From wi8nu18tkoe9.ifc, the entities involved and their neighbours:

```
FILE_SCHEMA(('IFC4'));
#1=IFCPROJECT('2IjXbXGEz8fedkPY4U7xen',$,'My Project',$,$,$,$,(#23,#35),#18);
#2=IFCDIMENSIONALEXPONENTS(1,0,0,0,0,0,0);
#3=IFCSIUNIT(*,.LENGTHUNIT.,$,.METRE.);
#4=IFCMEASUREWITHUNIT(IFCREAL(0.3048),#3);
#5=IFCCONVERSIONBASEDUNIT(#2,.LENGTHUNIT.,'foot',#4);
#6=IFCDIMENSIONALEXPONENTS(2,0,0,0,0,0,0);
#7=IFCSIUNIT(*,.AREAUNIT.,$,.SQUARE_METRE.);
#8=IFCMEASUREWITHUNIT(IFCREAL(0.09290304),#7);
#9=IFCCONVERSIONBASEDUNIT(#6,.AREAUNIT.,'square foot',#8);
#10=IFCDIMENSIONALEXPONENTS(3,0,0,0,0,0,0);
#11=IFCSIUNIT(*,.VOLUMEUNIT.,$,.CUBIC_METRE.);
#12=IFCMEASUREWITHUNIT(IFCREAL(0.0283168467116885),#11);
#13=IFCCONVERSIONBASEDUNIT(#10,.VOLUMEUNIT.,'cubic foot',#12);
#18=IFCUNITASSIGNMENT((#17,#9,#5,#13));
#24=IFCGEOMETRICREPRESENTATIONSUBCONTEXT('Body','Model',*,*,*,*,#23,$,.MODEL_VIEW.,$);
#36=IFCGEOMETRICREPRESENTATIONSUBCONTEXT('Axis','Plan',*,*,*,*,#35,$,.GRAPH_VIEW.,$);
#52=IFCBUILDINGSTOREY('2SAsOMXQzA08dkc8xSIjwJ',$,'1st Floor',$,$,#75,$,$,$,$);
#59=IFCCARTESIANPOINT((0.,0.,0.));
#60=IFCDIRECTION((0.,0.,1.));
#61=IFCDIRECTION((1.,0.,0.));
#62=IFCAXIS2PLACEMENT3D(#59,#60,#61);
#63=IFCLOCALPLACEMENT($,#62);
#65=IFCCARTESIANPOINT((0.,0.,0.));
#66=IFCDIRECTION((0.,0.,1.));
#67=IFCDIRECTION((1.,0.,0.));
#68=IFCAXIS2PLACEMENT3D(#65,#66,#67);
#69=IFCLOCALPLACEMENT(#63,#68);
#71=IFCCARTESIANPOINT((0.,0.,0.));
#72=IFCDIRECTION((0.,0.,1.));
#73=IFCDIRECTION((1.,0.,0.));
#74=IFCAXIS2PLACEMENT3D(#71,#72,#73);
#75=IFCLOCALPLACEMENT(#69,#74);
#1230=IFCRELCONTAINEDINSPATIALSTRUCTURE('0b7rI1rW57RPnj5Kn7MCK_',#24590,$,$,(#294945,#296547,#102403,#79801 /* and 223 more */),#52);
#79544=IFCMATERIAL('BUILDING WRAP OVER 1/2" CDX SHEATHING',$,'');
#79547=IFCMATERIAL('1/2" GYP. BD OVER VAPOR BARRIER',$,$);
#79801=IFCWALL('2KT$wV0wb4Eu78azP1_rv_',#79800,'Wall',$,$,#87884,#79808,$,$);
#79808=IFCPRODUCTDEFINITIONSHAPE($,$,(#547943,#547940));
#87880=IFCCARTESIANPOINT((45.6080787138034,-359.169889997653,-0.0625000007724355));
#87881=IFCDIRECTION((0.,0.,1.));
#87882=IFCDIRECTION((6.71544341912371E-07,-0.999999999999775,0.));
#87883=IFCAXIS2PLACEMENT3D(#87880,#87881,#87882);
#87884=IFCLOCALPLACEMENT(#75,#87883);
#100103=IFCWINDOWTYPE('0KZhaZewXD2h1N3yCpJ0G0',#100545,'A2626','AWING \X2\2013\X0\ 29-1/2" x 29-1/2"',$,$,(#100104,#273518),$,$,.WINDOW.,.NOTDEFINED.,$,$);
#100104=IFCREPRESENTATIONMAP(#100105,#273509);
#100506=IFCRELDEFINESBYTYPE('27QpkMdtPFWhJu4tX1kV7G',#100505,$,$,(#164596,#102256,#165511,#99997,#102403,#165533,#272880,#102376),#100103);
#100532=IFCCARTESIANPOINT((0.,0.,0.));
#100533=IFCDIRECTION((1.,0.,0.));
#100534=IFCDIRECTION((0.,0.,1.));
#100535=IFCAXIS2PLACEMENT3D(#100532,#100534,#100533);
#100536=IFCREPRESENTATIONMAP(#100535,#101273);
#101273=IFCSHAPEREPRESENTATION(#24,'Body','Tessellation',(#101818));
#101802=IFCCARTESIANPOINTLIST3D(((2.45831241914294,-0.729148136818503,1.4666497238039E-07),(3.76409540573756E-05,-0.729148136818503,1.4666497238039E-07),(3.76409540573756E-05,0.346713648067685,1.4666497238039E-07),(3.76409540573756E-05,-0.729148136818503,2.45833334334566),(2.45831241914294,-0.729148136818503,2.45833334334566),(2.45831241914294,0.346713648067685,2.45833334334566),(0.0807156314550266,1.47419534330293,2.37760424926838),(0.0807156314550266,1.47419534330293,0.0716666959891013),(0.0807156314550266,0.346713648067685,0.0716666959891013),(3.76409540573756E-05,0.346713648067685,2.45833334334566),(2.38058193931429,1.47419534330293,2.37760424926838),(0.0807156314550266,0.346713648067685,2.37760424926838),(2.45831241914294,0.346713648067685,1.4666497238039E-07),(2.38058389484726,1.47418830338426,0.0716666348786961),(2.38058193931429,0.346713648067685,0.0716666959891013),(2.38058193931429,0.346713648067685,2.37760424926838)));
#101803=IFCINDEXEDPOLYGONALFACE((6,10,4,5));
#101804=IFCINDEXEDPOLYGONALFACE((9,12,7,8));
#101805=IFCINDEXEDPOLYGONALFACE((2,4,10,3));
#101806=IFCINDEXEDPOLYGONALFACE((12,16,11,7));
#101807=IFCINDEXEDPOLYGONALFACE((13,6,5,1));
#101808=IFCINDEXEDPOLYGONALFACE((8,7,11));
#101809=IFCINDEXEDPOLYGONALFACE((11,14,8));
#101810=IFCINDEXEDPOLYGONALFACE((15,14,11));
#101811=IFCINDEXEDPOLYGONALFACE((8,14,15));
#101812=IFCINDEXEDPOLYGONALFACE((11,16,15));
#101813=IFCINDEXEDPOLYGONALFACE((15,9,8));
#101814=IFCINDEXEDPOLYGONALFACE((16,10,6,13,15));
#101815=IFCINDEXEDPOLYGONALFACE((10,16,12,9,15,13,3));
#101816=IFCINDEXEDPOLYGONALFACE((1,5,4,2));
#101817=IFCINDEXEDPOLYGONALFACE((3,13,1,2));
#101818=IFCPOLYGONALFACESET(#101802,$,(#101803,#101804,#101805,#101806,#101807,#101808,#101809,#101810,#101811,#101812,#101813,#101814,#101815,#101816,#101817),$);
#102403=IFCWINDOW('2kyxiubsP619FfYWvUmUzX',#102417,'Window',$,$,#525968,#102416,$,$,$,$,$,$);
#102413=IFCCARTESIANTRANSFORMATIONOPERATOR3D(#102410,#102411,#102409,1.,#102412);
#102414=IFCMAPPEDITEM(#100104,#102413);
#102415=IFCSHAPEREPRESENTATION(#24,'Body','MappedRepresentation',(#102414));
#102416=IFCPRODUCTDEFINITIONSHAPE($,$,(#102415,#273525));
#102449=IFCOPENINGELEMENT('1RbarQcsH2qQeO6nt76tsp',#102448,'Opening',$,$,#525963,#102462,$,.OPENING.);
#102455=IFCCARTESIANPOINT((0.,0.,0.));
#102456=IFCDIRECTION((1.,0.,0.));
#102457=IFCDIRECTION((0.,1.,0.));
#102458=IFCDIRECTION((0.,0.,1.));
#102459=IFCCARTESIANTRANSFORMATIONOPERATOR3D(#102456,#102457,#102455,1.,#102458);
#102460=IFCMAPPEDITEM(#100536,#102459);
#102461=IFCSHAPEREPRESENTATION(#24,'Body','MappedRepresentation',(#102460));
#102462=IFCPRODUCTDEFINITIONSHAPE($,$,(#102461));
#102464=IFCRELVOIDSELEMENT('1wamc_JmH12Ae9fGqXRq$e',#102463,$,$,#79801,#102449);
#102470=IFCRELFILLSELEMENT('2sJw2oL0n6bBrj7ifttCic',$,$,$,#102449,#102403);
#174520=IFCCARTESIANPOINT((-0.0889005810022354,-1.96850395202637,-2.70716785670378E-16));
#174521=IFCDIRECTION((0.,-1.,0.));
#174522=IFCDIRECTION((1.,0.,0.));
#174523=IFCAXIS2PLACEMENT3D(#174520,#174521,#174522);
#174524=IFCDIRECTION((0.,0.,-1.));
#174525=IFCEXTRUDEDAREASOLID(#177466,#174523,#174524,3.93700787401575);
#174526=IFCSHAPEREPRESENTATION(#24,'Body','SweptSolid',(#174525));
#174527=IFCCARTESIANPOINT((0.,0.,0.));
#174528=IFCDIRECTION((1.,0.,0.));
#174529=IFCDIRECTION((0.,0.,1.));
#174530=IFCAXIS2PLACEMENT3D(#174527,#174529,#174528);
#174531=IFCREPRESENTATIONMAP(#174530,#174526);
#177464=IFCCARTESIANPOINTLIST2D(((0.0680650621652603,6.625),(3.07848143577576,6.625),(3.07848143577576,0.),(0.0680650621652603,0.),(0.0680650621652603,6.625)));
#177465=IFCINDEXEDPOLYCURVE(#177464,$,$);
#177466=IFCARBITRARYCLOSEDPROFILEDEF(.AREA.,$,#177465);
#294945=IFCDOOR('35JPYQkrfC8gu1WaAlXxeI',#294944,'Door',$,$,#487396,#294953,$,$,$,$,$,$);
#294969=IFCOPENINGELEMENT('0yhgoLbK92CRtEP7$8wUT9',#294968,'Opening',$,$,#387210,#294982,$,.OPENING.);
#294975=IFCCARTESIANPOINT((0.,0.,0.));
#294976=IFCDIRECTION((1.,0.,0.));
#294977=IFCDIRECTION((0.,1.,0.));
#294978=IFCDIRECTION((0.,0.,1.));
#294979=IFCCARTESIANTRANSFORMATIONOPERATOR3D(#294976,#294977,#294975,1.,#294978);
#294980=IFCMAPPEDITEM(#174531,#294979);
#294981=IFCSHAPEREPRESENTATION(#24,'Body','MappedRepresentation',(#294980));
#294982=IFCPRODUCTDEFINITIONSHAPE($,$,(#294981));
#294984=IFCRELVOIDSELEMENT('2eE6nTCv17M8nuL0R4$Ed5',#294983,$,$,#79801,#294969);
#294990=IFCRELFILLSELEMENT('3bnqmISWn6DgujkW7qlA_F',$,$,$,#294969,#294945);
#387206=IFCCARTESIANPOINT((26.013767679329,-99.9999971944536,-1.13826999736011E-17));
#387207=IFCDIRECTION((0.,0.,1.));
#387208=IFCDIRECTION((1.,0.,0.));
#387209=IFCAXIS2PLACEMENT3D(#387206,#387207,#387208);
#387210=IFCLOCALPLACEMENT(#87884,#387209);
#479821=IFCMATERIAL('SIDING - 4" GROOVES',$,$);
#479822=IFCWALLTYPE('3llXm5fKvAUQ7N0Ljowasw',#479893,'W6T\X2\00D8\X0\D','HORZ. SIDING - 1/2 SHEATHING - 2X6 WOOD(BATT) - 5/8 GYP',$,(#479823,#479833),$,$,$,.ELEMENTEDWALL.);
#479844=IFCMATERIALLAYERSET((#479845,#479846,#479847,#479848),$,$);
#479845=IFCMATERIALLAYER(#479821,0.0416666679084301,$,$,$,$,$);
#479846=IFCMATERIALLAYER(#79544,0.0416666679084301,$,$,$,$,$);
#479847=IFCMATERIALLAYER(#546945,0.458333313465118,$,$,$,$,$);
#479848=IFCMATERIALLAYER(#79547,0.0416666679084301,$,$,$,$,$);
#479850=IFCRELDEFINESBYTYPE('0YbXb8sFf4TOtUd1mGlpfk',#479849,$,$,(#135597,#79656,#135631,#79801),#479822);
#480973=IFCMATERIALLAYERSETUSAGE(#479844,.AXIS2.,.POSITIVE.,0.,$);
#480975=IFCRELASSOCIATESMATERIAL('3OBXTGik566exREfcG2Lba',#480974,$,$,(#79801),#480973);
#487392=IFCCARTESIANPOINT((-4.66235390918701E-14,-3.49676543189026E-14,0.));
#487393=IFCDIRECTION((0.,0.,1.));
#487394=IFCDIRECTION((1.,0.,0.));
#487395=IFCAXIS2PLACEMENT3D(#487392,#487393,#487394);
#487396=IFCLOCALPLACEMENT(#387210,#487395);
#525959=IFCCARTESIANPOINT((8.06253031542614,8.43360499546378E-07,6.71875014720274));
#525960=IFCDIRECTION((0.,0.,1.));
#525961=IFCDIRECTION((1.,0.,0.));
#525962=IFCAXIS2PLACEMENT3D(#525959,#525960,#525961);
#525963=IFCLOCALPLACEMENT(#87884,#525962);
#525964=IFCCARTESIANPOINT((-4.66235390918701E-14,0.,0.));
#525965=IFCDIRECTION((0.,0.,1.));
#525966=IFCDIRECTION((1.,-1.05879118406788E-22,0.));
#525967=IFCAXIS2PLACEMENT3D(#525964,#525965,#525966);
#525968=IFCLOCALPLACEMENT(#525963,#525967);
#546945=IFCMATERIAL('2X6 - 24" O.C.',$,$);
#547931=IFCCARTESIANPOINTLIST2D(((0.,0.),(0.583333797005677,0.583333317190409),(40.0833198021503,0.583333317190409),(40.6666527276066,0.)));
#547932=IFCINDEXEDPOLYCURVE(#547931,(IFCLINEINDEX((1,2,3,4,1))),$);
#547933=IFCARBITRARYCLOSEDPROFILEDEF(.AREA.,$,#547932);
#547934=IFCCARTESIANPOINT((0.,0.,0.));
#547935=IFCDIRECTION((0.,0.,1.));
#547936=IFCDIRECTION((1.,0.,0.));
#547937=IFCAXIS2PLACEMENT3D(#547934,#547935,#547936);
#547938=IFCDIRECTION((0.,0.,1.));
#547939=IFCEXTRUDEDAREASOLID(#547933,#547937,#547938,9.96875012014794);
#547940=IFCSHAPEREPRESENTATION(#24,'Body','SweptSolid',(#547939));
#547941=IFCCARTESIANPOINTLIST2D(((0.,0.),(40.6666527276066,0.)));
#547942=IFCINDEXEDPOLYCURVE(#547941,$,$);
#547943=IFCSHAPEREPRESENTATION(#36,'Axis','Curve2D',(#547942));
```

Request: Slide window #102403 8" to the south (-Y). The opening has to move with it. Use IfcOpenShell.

```python
import ifcopenshell
import ifcopenshell.api.geometry
import ifcopenshell.util.placement
import ifcopenshell.util.unit

model = ifcopenshell.open("wi8nu18tkoe9.ifc")
unit_scale = ifcopenshell.util.unit.calculate_unit_scale(model)

window = model.by_guid("2kyxiubsP619FfYWvUmUzX")
opening = window.FillsVoids[0].RelatingOpeningElement
wall = opening.VoidsElements[0].RelatingBuildingElement

wall_matrix = ifcopenshell.util.placement.get_local_placement(wall.ObjectPlacement)
shift = wall_matrix[:3, 0] * 8 * 0.0254 / unit_scale
before = ifcopenshell.util.placement.get_local_placement(window.ObjectPlacement)[:3, 3].copy()

# The window is placed relative to its opening, so it follows when the opening moves.
matrix = ifcopenshell.util.placement.get_local_placement(opening.ObjectPlacement)
matrix[:3, 3] += shift
ifcopenshell.api.geometry.edit_object_placement(
    model, product=opening, matrix=matrix, is_si=False, should_transform_children=True
)

after = ifcopenshell.util.placement.get_local_placement(window.ObjectPlacement)[:3, 3]
print("window moved by", (after - before).round(3) + 0.0)

model.write("wi8nu18tkoe9-out.ifc")
```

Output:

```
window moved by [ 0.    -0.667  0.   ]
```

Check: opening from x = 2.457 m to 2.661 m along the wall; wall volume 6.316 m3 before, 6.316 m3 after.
